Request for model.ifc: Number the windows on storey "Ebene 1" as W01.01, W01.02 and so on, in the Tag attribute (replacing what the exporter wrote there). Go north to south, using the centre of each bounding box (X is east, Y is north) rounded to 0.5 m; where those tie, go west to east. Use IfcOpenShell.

First a look at what the model holds.

```python
import ifcopenshell
import ifcopenshell.util.element
import ifcopenshell.util.placement

model = ifcopenshell.open("model.ifc")
print(model.schema)
storey = next(s for s in model.by_type("IfcBuildingStorey") if s.Name == "Ebene 1")
windows = [e for e in ifcopenshell.util.element.get_decomposition(storey) if e.is_a("IfcWindow")]
for e in sorted(windows, key=lambda e: e.id()):
    origin = ifcopenshell.util.placement.get_local_placement(e.ObjectPlacement)[:3, 3]
    print(e.id(), e.Tag, e.Name, origin.round(2) + 0.0, sep=" | ")
```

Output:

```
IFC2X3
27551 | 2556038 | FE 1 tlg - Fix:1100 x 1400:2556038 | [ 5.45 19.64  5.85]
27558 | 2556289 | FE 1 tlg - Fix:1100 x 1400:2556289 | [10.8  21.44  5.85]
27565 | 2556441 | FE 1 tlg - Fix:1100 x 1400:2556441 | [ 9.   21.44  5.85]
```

```python
import ifcopenshell
import ifcopenshell.geom
import ifcopenshell.util.element
import ifcopenshell.util.shape

model = ifcopenshell.open("model.ifc")
settings = ifcopenshell.geom.settings()
settings.set("use-world-coords", True)


def centre(element):
    shape = ifcopenshell.geom.create_shape(settings, element)
    return ifcopenshell.util.shape.get_bbox_centroid(shape.geometry)


storey = next(s for s in model.by_type("IfcBuildingStorey") if s.Name == "Ebene 1")
windows = [e for e in ifcopenshell.util.element.get_decomposition(storey) if e.is_a("IfcWindow")]

# Insertion points can sit at a corner or the storey origin, so sort by the geometry (in metres).
centres = {e: centre(e) for e in windows}
windows.sort(key=lambda e: (-round(centres[e][1] / 0.5), centres[e][0]))

for i, e in enumerate(windows, start=1):
    number = f"W01.{i:02d}"
    e.Tag = number
    print(e.id(), number)

model.write("model_updated.ifc")
```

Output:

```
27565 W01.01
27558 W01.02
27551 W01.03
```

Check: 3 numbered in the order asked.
